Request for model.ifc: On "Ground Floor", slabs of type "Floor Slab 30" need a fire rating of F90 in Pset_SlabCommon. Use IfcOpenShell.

First a look at what the model holds.

```python
import ifcopenshell
import ifcopenshell.util.element

model = ifcopenshell.open("model.ifc")
print(model.schema)
storey = next(s for s in model.by_type("IfcBuildingStorey") if s.Name == "Ground Floor")
slabs = [e for e in ifcopenshell.util.element.get_decomposition(storey) if e.is_a("IfcSlab")]
seen = {}
for e in slabs:
    element_type = ifcopenshell.util.element.get_type(e)
    key = (element_type.Name if element_type != e and element_type else None, ifcopenshell.util.element.get_pset(e, "Pset_SlabCommon", "FireRating"))
    seen[key] = seen.get(key, 0) + 1
for (name, value), count in sorted(seen.items(), key=str):
    print(count, "x", name, "|", value)
```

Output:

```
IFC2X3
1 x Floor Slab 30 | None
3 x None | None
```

```python
import ifcopenshell
import ifcopenshell.api.pset
import ifcopenshell.util.element

model = ifcopenshell.open("model.ifc")

storey = next(s for s in model.by_type("IfcBuildingStorey") if s.Name == "Ground Floor")
slabs = [e for e in ifcopenshell.util.element.get_decomposition(storey) if e.is_a("IfcSlab")]

count = 0
for e in slabs:
    element_type = ifcopenshell.util.element.get_type(e)
    if element_type in (None, e) or element_type.Name != "Floor Slab 30":
        continue
    # add_pset returns the element's existing set when there is one.
    pset = ifcopenshell.api.pset.add_pset(model, product=e, name="Pset_SlabCommon")
    ifcopenshell.api.pset.edit_pset(model, pset=pset, properties={"FireRating": "F90"})
    count += 1

print(count, "slabs updated")

model.write("model_edited.ifc")
```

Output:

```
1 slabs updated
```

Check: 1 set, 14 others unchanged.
